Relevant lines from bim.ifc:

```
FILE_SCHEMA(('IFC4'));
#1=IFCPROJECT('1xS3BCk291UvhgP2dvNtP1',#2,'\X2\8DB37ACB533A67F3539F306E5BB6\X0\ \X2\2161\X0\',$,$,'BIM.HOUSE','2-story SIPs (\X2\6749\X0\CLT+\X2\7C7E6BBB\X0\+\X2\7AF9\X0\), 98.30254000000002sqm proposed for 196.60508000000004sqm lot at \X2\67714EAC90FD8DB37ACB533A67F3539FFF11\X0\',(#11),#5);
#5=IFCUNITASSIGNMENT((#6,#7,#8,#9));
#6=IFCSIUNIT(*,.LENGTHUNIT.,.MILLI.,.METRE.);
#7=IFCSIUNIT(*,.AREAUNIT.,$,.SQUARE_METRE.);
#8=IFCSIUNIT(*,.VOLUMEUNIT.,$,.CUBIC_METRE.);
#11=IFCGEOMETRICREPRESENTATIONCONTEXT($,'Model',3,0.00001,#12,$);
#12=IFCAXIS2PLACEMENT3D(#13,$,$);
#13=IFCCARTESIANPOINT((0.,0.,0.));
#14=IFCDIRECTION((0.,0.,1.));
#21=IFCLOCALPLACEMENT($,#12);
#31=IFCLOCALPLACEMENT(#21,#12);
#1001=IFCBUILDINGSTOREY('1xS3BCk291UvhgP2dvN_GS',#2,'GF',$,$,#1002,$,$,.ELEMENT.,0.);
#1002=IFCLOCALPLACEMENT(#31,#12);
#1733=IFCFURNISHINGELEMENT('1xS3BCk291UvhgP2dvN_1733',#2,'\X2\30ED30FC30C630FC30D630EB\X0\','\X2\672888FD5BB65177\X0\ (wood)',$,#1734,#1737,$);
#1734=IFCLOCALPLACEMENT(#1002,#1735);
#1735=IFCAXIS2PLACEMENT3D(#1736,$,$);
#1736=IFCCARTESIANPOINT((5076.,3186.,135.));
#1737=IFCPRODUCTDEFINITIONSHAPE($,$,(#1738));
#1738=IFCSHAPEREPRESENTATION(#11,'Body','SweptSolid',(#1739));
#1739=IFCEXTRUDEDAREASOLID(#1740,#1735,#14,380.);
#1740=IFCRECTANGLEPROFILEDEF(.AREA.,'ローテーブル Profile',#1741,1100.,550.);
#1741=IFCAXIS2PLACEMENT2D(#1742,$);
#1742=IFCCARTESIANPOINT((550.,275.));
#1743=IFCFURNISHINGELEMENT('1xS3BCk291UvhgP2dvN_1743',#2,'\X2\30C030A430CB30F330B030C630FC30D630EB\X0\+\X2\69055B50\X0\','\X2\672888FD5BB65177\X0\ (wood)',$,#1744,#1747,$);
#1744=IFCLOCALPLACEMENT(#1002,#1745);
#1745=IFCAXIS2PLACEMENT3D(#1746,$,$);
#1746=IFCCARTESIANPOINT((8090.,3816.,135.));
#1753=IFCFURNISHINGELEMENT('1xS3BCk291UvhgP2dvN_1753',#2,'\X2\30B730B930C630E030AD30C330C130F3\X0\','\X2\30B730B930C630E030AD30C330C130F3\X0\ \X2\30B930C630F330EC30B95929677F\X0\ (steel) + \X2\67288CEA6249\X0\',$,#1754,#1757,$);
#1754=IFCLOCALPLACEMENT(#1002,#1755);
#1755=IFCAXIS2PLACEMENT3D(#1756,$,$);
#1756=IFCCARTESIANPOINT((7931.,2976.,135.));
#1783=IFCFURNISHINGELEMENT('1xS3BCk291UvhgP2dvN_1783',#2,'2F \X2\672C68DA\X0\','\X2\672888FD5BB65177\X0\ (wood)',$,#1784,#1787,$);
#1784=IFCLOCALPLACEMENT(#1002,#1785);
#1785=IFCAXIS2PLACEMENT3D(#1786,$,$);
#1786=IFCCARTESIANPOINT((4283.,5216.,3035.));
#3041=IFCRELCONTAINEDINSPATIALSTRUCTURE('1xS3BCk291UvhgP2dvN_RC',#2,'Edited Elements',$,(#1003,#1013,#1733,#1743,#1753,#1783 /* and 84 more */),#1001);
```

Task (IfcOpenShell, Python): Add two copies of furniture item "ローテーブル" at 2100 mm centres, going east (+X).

```python
import numpy as np
import ifcopenshell
import ifcopenshell.api.geometry
import ifcopenshell.api.root
import ifcopenshell.util.element
import ifcopenshell.util.placement

model = ifcopenshell.open("bim.ifc")


def reuse_history(source, copy):
    """copy_class also copies each property set's owner history, people and application; keep the originals."""
    for rel in copy.IsDefinedBy:
        if rel.is_a("IfcRelDefinesByProperties") and (history := rel.RelatingPropertyDefinition.OwnerHistory):
            rel.RelatingPropertyDefinition.OwnerHistory = source.OwnerHistory
            ifcopenshell.util.element.remove_deep2(model, history)


source = model.by_id(1733)
base = ifcopenshell.util.placement.get_local_placement(source.ObjectPlacement)
step = np.array([1.0, 0.0, 0.0]) * 2100.0

for i in range(1, 3):
    copy = ifcopenshell.api.root.copy_class(model, product=source)
    copy.Representation = ifcopenshell.util.element.copy_deep(
        model, source.Representation, exclude=["IfcGeometricRepresentationContext", "IfcRepresentationMap"]
    )
    reuse_history(source, copy)
    matrix = base.copy()
    matrix[:3, 3] += i * step
    print("added at", matrix[:3, 3].round(3) + 0.0)
    ifcopenshell.api.geometry.edit_object_placement(model, product=copy, matrix=matrix, is_si=False)

model.write("bim_rev.ifc")
```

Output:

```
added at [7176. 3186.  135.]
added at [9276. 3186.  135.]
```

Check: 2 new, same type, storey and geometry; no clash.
